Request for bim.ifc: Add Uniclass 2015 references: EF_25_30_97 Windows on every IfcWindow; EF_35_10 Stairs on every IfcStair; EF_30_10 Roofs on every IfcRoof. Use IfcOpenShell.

First a look at what the model holds.

```python
import ifcopenshell

model = ifcopenshell.open("bim.ifc")
print(model.schema)
print("classifications:", [c.Name for c in model.by_type("IfcClassification")])
for ifc_class in ("IfcDoor", "IfcRoof", "IfcStair", "IfcWall", "IfcWindow"):
    print(ifc_class, len(model.by_type(ifc_class)))
```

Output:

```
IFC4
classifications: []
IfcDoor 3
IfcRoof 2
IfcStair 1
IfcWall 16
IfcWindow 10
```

```python
import ifcopenshell
import ifcopenshell.api.classification

model = ifcopenshell.open("bim.ifc")

system = ifcopenshell.api.classification.add_classification(model, classification="Uniclass 2015")

codes = {
    "IfcWindow": ("EF_25_30_97", "Windows"),
    "IfcStair": ("EF_35_10", "Stairs"),
    "IfcRoof": ("EF_30_10", "Roofs"),
}
for ifc_class, (code, name) in codes.items():
    products = model.by_type(ifc_class)
    ifcopenshell.api.classification.add_reference(
        model, products=products, classification=system, identification=code, name=name
    )
    print(code, len(products))

model.write("bim-out.ifc")
```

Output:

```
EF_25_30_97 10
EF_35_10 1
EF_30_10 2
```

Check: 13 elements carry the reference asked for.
